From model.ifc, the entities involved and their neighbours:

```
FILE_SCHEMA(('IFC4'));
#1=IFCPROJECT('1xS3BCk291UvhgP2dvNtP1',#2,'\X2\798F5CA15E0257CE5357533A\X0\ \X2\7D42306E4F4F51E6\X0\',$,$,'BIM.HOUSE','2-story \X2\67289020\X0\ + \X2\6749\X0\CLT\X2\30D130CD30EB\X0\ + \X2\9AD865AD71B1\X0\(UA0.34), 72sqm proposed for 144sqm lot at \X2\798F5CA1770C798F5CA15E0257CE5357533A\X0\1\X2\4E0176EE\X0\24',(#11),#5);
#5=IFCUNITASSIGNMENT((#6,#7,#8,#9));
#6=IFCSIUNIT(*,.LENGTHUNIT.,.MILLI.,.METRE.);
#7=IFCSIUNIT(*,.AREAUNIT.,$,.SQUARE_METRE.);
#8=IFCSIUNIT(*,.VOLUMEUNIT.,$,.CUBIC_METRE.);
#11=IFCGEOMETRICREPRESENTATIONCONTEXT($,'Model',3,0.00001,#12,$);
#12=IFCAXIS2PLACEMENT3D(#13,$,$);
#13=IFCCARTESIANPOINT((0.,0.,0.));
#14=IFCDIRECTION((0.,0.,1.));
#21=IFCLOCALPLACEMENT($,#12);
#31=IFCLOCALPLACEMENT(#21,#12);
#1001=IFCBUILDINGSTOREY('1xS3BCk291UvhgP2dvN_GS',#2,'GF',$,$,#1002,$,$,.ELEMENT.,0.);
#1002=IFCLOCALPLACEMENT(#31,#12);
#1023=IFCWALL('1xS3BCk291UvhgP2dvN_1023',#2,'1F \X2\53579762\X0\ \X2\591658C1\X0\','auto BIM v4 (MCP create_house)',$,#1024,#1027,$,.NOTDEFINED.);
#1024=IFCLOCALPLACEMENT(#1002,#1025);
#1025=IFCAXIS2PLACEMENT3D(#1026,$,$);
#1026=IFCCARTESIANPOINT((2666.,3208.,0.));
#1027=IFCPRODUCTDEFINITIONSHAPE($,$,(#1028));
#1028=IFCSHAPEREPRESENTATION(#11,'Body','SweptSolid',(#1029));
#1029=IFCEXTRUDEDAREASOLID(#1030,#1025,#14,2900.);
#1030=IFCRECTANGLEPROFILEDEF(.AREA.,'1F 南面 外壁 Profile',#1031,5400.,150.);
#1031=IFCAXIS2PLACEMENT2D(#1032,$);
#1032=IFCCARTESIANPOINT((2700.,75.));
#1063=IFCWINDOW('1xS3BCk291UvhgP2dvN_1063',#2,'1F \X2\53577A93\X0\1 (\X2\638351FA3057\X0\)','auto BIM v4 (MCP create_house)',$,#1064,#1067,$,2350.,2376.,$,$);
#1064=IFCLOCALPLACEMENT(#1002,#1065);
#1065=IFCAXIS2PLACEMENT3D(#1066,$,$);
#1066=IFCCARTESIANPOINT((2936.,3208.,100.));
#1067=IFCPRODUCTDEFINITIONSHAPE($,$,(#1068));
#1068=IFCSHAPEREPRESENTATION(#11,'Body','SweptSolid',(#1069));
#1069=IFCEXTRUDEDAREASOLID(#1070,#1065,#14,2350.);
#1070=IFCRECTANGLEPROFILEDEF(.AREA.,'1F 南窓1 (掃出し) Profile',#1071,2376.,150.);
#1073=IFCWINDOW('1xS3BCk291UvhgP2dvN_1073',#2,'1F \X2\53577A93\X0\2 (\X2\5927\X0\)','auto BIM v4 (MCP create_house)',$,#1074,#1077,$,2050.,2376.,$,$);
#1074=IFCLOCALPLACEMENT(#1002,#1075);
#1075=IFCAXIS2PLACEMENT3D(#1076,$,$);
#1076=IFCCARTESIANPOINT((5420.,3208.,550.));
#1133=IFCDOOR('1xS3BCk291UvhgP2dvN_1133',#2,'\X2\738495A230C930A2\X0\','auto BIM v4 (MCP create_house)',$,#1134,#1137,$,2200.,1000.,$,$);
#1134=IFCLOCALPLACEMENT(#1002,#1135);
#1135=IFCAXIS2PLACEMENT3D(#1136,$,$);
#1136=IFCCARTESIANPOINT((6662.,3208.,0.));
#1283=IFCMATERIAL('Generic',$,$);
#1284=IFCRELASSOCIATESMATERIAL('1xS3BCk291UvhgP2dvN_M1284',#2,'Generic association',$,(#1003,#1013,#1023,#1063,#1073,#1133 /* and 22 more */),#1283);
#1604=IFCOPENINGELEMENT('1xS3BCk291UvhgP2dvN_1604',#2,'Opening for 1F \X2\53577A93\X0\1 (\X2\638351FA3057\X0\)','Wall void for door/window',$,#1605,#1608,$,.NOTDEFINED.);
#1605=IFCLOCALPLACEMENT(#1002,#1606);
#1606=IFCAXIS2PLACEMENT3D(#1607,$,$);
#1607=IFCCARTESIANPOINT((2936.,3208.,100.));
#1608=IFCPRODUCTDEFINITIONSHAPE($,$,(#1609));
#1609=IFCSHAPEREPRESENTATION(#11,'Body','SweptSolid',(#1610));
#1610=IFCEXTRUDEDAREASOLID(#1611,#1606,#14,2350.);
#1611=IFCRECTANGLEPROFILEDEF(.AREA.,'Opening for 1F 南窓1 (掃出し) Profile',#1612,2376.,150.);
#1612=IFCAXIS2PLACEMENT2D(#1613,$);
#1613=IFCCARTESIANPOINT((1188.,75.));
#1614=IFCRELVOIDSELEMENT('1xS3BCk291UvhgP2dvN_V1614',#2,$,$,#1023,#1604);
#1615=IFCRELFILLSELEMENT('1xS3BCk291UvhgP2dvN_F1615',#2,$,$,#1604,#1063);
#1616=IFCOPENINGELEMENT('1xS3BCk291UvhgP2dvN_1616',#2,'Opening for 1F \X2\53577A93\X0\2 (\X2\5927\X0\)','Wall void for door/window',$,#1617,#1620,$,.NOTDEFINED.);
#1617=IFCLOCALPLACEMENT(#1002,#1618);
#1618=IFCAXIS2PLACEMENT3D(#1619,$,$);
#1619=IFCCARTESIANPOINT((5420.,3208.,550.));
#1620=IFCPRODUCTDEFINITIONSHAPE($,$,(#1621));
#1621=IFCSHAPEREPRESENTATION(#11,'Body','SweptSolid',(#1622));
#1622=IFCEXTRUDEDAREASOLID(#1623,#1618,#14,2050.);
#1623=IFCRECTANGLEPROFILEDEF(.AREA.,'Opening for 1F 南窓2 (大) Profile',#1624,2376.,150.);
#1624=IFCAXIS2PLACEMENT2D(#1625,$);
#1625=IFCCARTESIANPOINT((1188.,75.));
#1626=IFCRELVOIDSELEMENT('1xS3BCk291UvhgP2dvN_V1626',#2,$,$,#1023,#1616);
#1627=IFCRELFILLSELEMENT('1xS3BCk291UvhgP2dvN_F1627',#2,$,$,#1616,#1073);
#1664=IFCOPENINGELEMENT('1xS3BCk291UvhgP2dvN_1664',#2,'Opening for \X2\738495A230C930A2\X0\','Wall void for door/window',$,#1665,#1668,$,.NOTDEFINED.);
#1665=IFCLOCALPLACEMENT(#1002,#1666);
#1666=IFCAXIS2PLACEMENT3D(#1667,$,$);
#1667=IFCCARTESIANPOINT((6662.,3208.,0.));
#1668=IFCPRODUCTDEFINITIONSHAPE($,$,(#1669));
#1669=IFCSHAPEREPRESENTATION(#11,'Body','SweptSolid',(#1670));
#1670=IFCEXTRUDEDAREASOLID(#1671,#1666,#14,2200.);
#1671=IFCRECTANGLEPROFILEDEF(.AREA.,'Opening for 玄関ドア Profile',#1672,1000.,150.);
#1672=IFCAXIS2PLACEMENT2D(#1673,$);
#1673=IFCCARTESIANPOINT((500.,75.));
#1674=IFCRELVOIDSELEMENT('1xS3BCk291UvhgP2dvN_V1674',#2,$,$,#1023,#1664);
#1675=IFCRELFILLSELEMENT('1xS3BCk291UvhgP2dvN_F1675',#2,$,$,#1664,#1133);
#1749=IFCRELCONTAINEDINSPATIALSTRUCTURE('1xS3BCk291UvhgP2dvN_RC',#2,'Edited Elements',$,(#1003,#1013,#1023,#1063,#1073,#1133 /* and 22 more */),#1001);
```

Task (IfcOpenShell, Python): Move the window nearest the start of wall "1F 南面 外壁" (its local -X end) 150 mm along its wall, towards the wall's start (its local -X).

```python
import ifcopenshell
import ifcopenshell.api.geometry
import ifcopenshell.util.placement

model = ifcopenshell.open("model.ifc")

window = model.by_guid("1xS3BCk291UvhgP2dvN_1063")
opening = window.FillsVoids[0].RelatingOpeningElement
wall = opening.VoidsElements[0].RelatingBuildingElement

wall_matrix = ifcopenshell.util.placement.get_local_placement(wall.ObjectPlacement)
shift = wall_matrix[:3, 0] * -150.0
before = ifcopenshell.util.placement.get_local_placement(window.ObjectPlacement)[:3, 3].copy()

# The window is not placed relative to its opening, so move both.
for product in (opening, window):
    matrix = ifcopenshell.util.placement.get_local_placement(product.ObjectPlacement)
    matrix[:3, 3] += shift
    ifcopenshell.api.geometry.edit_object_placement(model, product=product, matrix=matrix, is_si=False)

after = ifcopenshell.util.placement.get_local_placement(window.ObjectPlacement)[:3, 3]
print("window moved by", (after - before).round(3) + 0.0)

model.write("model-out.ifc")
```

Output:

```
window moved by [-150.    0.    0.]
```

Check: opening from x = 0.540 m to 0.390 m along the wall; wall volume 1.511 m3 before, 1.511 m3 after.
